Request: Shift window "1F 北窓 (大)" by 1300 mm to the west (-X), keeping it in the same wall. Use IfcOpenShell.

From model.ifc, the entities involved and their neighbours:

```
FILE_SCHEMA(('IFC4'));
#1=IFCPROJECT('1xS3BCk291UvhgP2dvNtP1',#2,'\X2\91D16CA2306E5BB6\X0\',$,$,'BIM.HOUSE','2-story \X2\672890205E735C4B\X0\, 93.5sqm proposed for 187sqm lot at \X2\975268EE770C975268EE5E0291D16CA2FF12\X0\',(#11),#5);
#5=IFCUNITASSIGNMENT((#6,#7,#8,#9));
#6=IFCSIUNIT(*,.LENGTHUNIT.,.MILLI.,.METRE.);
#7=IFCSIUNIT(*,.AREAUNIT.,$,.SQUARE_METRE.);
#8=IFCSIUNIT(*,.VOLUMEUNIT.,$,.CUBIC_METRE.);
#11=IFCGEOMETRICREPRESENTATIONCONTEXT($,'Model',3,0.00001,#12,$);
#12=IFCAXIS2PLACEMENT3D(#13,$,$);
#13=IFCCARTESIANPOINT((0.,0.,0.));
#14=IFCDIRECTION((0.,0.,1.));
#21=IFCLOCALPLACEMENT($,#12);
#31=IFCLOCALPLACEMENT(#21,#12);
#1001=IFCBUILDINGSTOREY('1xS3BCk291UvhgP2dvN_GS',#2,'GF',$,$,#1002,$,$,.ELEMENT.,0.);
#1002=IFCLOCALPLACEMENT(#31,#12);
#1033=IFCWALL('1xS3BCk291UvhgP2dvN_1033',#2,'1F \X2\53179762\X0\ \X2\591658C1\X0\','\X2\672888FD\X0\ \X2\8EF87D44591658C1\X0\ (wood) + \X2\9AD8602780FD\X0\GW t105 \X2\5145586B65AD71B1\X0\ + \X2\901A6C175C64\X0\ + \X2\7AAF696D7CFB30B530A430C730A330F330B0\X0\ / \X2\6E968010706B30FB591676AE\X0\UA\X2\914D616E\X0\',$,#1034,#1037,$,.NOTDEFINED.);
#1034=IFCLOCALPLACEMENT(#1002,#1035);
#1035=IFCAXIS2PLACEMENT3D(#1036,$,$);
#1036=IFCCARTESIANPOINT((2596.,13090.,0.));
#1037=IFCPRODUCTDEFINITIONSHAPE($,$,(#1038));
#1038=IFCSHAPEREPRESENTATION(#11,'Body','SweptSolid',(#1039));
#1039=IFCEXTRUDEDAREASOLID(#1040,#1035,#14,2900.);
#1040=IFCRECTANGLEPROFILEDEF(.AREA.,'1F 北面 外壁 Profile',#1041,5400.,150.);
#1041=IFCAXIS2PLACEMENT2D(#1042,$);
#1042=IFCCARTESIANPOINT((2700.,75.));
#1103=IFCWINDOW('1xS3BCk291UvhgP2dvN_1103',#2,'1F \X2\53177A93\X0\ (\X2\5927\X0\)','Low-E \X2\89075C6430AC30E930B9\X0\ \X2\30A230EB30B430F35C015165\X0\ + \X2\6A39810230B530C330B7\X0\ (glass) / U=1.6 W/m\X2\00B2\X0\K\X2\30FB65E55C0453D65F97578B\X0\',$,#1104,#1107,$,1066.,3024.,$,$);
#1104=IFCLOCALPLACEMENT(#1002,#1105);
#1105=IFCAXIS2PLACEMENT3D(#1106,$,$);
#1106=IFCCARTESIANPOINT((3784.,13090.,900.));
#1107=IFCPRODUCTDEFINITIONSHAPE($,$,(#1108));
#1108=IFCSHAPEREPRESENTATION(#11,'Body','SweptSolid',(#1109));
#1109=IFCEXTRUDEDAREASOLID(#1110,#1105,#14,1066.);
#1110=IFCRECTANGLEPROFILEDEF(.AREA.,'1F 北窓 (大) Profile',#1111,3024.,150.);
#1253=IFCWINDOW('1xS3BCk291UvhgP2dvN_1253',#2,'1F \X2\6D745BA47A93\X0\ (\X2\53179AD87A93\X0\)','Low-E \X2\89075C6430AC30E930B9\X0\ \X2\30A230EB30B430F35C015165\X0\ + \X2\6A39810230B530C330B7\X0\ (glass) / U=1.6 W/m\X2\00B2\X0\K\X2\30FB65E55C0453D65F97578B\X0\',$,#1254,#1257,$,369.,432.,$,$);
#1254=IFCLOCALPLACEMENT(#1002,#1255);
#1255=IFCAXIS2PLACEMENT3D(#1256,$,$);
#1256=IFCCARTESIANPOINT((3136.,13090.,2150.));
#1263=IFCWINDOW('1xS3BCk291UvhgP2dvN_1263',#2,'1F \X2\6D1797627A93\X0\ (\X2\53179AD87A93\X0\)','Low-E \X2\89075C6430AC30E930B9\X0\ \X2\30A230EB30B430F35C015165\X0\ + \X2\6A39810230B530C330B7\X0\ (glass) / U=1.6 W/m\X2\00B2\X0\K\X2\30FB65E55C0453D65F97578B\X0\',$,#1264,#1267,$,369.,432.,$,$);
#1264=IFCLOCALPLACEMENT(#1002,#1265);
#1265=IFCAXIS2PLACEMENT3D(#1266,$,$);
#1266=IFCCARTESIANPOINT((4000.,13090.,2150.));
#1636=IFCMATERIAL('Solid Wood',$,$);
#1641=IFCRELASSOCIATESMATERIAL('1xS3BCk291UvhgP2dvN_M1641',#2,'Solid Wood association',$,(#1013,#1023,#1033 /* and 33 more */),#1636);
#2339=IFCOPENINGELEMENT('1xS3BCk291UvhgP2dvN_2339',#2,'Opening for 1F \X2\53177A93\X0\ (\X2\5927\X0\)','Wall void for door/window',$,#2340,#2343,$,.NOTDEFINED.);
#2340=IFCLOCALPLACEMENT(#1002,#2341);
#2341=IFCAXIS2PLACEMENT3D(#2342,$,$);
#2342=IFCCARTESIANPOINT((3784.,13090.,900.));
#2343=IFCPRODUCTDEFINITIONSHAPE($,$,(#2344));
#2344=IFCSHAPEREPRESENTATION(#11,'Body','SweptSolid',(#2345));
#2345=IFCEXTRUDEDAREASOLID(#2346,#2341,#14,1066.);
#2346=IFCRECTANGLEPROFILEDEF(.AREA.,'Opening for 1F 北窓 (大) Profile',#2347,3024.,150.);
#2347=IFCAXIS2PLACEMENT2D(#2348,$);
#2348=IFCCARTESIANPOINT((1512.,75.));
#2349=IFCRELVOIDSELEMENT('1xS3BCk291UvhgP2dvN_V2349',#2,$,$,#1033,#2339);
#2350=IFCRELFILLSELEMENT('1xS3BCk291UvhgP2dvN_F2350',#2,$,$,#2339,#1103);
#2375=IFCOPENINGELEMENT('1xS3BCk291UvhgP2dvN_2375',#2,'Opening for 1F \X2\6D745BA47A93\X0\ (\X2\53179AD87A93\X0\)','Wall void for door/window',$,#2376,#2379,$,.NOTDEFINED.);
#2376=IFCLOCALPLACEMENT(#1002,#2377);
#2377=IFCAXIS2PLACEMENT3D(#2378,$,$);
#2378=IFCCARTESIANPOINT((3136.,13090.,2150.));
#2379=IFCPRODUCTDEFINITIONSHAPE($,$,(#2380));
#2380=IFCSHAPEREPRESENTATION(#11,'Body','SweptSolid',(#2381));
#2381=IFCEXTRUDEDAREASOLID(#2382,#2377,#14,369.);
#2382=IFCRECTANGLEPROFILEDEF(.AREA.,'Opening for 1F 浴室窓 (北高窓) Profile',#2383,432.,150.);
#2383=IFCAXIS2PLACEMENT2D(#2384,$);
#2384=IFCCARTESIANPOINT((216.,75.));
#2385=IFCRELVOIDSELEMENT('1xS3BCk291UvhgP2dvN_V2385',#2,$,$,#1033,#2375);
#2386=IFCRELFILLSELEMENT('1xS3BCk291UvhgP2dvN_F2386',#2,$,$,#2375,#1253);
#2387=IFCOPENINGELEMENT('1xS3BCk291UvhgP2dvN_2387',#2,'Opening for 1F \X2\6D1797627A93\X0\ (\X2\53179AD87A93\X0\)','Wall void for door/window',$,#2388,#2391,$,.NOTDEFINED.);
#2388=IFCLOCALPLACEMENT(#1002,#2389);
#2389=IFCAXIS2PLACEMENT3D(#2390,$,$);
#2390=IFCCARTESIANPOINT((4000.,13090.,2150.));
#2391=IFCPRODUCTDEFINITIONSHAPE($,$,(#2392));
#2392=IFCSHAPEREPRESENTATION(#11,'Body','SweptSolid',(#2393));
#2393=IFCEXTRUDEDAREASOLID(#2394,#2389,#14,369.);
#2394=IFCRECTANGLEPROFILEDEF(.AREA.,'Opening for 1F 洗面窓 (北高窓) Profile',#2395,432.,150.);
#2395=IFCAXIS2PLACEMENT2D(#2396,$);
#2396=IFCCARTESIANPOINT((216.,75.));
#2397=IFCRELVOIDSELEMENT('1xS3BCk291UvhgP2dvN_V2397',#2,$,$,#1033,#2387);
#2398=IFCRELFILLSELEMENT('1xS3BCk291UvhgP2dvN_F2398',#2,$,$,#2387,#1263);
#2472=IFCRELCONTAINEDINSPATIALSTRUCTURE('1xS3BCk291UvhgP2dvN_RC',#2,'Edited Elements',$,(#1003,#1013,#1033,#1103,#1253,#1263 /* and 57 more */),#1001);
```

```python
import ifcopenshell
import ifcopenshell.api.geometry
import ifcopenshell.util.placement
import ifcopenshell.util.unit

model = ifcopenshell.open("model.ifc")
unit_scale = ifcopenshell.util.unit.calculate_unit_scale(model)

window = model.by_guid("1xS3BCk291UvhgP2dvN_1103")
opening = window.FillsVoids[0].RelatingOpeningElement
wall = opening.VoidsElements[0].RelatingBuildingElement

wall_matrix = ifcopenshell.util.placement.get_local_placement(wall.ObjectPlacement)
shift = wall_matrix[:3, 0] * -1.3 / unit_scale
before = ifcopenshell.util.placement.get_local_placement(window.ObjectPlacement)[:3, 3].copy()

# The window is not placed relative to its opening, so move both.
for product in (opening, window):
    matrix = ifcopenshell.util.placement.get_local_placement(product.ObjectPlacement)
    matrix[:3, 3] += shift
    ifcopenshell.api.geometry.edit_object_placement(model, product=product, matrix=matrix, is_si=False)

after = ifcopenshell.util.placement.get_local_placement(window.ObjectPlacement)[:3, 3]
print("window moved by", (after - before).round(3) + 0.0)

model.write("model_updated.ifc")
```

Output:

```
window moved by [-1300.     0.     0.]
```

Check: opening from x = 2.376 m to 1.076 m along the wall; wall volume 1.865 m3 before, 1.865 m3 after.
